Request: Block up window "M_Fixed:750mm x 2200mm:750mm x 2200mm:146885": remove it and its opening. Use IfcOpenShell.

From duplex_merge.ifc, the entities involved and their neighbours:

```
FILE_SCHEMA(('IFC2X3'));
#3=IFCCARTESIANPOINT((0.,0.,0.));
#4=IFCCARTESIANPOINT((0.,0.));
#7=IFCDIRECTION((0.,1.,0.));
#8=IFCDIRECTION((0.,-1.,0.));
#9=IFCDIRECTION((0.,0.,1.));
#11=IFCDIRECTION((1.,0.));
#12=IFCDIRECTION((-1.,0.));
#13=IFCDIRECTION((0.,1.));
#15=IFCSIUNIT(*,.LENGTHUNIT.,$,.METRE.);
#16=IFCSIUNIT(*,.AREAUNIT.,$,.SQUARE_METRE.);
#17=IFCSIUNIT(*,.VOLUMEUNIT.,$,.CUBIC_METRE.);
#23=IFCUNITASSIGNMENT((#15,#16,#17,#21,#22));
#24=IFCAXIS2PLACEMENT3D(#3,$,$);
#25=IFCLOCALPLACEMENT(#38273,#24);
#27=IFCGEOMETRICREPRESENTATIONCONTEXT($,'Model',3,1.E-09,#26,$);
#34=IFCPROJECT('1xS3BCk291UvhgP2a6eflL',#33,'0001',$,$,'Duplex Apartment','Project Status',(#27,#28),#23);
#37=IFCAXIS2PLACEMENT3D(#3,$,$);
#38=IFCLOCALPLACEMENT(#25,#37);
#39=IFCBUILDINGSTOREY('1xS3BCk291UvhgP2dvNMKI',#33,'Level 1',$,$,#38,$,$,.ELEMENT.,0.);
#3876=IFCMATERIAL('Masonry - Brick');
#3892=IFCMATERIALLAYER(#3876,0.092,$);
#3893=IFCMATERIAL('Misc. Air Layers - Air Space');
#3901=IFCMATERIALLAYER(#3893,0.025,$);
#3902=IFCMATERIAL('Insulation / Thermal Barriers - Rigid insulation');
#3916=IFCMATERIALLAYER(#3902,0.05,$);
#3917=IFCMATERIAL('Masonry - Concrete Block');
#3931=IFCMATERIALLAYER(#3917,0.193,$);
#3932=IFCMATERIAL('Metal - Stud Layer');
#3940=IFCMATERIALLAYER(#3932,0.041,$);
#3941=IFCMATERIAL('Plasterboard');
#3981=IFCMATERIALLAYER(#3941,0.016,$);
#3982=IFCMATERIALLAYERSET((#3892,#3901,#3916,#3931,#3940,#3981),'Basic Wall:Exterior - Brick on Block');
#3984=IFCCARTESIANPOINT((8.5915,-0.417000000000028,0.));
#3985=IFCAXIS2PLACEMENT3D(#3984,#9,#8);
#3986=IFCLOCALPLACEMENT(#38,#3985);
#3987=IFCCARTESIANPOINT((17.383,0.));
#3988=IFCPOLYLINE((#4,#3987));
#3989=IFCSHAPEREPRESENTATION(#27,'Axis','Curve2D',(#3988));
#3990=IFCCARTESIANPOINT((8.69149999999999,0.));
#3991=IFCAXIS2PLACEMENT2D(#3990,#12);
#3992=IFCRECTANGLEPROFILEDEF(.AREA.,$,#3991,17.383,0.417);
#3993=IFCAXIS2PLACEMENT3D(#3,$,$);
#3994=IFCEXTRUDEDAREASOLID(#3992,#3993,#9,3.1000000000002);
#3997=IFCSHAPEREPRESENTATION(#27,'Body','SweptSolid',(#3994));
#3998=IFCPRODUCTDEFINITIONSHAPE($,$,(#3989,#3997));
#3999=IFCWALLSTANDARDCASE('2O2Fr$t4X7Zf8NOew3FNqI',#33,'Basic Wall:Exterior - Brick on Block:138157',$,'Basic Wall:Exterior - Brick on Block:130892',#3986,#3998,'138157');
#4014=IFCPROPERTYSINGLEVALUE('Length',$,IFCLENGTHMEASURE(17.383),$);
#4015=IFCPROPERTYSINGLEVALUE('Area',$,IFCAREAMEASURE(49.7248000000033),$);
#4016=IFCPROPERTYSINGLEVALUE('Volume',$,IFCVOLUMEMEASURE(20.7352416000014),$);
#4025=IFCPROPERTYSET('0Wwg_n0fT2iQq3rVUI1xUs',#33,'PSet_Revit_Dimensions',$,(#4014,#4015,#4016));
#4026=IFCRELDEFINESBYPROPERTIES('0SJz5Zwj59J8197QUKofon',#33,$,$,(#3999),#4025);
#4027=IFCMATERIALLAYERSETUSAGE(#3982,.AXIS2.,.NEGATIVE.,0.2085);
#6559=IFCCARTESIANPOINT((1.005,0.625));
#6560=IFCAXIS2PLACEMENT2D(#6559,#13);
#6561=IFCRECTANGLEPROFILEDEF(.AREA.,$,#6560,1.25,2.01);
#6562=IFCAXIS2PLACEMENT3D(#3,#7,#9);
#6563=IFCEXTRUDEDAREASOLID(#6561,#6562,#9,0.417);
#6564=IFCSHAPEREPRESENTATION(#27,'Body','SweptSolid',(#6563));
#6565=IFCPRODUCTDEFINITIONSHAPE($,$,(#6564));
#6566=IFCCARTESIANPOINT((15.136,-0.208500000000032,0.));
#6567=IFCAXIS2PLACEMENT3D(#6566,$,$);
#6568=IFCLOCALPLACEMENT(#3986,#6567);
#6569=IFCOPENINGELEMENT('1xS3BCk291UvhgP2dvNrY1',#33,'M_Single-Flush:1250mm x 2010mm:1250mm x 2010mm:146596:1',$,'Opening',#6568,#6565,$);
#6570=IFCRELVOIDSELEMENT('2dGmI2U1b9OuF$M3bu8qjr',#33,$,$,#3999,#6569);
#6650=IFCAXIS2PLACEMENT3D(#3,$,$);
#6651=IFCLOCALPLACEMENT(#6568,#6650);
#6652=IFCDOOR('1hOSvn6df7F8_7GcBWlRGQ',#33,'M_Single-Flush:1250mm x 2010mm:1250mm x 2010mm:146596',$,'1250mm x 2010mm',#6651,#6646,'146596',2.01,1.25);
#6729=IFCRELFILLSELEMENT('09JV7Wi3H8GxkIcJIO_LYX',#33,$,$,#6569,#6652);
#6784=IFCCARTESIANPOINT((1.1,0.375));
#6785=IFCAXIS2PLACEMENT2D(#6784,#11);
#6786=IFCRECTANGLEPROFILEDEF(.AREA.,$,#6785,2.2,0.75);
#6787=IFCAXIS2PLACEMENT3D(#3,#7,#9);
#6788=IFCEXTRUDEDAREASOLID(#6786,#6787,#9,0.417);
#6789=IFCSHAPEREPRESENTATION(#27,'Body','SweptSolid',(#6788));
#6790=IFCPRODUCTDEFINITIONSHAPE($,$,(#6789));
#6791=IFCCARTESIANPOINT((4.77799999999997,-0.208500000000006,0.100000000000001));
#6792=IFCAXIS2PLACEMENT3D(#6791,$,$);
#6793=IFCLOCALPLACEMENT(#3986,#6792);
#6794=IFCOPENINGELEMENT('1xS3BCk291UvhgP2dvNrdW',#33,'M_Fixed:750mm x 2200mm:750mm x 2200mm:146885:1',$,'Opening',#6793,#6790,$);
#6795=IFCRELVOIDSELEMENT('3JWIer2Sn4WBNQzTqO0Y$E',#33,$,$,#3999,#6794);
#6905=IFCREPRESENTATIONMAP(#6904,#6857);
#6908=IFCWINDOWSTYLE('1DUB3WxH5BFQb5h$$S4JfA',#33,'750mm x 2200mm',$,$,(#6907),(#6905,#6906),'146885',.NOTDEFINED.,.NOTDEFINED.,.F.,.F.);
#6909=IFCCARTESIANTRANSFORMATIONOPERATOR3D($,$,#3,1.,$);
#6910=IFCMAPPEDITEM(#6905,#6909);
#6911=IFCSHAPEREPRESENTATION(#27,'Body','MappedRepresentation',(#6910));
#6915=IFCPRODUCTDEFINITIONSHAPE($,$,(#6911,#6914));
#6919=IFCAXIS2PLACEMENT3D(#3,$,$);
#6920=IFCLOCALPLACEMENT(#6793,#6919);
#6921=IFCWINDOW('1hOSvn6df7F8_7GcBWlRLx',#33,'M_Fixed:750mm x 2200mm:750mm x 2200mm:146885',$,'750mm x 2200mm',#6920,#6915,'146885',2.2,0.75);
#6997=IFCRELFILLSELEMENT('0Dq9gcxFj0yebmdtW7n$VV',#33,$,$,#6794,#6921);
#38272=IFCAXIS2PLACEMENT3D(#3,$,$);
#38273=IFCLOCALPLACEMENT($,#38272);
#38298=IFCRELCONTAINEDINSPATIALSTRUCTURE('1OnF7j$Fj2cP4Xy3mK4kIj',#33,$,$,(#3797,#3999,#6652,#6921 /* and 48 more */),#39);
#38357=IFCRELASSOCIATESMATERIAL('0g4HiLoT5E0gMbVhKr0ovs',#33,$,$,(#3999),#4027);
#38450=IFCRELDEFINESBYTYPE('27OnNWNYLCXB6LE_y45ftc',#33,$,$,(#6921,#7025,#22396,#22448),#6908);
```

```python
import ifcopenshell
import ifcopenshell.api.feature
import ifcopenshell.api.pset
import ifcopenshell.api.root
import ifcopenshell.geom
import ifcopenshell.util.element
import ifcopenshell.util.shape
import ifcopenshell.util.unit

model = ifcopenshell.open("duplex_merge.ifc")
area_scale = ifcopenshell.util.unit.calculate_unit_scale(model, "AREAUNIT")
volume_scale = ifcopenshell.util.unit.calculate_unit_scale(model, "VOLUMEUNIT")
settings = ifcopenshell.geom.settings()


def volume(element):
    """Net volume in cubic metres, openings subtracted."""
    shape = ifcopenshell.geom.create_shape(settings, element)
    return ifcopenshell.util.shape.get_volume(shape.geometry)


window = model.by_guid("1hOSvn6df7F8_7GcBWlRLx")
opening = window.FillsVoids[0].RelatingOpeningElement
wall = opening.VoidsElements[0].RelatingBuildingElement
before = volume(wall)

ifcopenshell.api.root.remove_product(model, product=window)
ifcopenshell.api.feature.remove_feature(model, feature=opening)

after = volume(wall)
thickness = 0.417  # wall thickness in metres

# Update the wall's stored quantities.
pset = model.by_id(ifcopenshell.util.element.get_pset(wall, "PSet_Revit_Dimensions", should_inherit=False)["id"])
ifcopenshell.api.pset.edit_pset(model, pset=pset, properties={
    "Area": model.create_entity("IfcAreaMeasure", after / thickness / area_scale),
    "Volume": model.create_entity("IfcVolumeMeasure", after / volume_scale),
})

print(f"wall volume {before:.3f} -> {after:.3f} m3")

model.write("duplex_merge_edited.ifc")
```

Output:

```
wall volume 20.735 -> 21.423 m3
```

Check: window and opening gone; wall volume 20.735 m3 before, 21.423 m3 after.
